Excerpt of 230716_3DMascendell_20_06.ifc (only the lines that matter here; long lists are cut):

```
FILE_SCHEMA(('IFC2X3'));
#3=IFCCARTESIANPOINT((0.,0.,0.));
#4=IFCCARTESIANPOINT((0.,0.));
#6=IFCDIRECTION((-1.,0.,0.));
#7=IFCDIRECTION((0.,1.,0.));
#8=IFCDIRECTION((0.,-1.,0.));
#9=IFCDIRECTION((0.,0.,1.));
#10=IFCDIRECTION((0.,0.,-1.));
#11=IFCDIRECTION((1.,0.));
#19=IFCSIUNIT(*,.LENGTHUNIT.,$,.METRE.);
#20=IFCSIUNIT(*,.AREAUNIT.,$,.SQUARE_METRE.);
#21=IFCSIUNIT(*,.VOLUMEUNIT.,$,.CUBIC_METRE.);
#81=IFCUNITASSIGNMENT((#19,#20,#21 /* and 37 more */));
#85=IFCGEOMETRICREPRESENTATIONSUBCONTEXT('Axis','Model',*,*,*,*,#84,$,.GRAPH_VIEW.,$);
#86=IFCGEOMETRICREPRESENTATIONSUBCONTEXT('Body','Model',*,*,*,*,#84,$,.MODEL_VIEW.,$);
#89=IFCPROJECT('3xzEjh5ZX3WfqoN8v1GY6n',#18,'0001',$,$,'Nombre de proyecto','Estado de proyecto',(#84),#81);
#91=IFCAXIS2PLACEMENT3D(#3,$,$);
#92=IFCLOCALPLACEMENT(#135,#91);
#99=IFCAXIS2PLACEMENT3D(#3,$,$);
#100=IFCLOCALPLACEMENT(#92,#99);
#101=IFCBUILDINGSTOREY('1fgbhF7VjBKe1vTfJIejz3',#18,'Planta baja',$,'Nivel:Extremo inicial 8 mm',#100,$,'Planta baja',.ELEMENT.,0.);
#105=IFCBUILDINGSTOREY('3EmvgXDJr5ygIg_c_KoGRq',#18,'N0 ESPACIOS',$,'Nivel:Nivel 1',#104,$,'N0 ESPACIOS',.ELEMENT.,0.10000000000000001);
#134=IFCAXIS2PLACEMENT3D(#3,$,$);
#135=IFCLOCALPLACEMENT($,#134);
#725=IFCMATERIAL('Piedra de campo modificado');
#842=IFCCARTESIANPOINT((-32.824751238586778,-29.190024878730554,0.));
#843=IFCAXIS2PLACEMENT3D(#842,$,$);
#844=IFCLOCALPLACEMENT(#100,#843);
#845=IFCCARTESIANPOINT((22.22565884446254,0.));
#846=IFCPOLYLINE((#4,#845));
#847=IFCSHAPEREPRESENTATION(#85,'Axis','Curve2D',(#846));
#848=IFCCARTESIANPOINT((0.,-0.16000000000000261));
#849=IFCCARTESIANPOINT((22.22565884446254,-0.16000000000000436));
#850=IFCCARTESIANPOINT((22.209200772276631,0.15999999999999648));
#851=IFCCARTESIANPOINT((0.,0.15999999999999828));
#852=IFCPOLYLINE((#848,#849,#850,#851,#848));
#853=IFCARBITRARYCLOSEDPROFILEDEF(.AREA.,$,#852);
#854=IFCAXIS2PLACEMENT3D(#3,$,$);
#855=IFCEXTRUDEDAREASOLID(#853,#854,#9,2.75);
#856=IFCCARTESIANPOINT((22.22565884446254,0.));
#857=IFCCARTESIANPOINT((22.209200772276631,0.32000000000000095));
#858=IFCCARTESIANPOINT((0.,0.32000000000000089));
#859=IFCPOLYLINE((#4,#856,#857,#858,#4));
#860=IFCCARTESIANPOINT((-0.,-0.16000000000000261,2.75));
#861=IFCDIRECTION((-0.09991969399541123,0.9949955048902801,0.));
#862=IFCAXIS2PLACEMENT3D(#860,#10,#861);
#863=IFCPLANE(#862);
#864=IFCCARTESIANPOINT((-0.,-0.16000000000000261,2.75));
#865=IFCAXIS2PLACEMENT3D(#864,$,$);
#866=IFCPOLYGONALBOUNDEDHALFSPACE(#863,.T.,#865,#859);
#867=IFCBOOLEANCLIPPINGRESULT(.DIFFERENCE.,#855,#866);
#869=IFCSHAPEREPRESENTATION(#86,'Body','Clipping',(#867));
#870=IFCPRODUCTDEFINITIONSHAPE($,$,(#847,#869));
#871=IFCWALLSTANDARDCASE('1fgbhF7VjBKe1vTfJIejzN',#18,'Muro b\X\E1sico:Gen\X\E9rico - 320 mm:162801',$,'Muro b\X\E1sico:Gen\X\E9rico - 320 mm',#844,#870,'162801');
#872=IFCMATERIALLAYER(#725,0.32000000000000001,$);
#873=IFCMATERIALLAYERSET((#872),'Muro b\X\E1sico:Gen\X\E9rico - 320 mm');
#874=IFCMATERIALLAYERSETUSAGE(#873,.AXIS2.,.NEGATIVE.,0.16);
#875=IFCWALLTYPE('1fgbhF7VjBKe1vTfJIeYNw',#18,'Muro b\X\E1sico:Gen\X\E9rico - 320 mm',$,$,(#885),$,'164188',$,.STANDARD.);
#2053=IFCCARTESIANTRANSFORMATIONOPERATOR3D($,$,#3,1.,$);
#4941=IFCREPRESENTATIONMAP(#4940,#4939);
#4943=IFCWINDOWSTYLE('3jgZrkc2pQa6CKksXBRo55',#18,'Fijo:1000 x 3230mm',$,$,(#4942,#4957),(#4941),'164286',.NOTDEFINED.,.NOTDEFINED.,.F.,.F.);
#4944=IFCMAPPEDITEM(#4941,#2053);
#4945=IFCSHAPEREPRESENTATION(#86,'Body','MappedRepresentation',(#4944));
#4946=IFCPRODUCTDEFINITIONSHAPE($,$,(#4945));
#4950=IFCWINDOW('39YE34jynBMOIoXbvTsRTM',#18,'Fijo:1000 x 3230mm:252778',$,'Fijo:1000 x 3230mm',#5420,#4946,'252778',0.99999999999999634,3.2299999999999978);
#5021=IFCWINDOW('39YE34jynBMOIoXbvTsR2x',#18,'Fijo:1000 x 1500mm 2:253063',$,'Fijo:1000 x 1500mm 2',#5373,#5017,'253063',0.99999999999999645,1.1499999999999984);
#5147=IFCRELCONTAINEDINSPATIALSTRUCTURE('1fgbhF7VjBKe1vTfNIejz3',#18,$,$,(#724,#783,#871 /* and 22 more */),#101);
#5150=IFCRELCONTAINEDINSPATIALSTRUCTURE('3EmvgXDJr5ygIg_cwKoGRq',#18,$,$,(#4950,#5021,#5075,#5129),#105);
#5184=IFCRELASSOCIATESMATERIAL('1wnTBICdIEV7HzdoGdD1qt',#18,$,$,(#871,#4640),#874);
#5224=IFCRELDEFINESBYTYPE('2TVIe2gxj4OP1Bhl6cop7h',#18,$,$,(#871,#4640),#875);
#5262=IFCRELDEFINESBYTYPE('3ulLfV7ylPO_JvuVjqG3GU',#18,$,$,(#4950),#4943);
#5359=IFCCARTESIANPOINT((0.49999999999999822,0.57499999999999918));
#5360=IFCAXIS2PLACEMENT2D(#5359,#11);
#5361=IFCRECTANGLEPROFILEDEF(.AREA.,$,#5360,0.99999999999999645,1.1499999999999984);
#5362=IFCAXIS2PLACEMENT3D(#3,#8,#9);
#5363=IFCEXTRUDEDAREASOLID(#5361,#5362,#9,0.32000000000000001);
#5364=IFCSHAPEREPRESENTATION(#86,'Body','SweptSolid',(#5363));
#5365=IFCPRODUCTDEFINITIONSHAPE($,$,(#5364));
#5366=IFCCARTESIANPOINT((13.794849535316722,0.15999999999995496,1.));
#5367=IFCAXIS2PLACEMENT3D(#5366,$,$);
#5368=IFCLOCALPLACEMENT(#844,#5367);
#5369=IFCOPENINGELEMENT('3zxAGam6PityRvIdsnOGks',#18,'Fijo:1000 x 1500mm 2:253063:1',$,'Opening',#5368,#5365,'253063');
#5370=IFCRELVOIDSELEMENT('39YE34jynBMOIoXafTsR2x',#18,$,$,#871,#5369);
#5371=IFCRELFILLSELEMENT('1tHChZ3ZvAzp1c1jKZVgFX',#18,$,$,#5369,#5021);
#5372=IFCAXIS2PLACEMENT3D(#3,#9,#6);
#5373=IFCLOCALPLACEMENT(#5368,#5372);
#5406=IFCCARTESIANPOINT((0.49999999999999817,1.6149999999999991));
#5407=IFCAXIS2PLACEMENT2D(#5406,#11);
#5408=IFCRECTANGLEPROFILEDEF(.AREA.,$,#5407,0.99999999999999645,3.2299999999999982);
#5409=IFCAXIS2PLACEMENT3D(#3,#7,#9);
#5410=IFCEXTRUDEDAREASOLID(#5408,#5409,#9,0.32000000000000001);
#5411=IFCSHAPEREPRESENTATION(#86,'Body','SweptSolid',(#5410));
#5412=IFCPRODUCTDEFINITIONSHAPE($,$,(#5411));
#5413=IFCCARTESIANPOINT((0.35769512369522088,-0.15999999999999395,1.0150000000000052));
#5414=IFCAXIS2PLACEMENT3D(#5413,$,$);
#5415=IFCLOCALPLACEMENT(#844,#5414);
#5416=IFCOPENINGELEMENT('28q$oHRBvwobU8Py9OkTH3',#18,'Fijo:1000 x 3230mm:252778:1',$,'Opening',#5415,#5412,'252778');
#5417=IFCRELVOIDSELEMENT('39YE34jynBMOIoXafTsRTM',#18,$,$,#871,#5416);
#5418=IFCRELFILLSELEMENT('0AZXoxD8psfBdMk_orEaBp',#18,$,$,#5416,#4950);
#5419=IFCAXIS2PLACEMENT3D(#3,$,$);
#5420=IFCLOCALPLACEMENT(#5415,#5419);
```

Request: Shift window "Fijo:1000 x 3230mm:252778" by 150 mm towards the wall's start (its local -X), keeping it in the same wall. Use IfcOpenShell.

```python
import ifcopenshell
import ifcopenshell.api.geometry
import ifcopenshell.util.placement
import ifcopenshell.util.unit

model = ifcopenshell.open("230716_3DMascendell_20_06.ifc")
unit_scale = ifcopenshell.util.unit.calculate_unit_scale(model)

window = model.by_guid("39YE34jynBMOIoXbvTsRTM")
opening = window.FillsVoids[0].RelatingOpeningElement
wall = opening.VoidsElements[0].RelatingBuildingElement

wall_matrix = ifcopenshell.util.placement.get_local_placement(wall.ObjectPlacement)
shift = wall_matrix[:3, 0] * -0.15 / unit_scale
before = ifcopenshell.util.placement.get_local_placement(window.ObjectPlacement)[:3, 3].copy()

# The window is placed relative to its opening, so it follows when the opening moves.
matrix = ifcopenshell.util.placement.get_local_placement(opening.ObjectPlacement)
matrix[:3, 3] += shift
ifcopenshell.api.geometry.edit_object_placement(
    model, product=opening, matrix=matrix, is_si=False, should_transform_children=True
)

after = ifcopenshell.util.placement.get_local_placement(window.ObjectPlacement)[:3, 3]
print("window moved by", (after - before).round(3) + 0.0)

model.write("230716_3DMascendell_20_06_updated.ifc")
```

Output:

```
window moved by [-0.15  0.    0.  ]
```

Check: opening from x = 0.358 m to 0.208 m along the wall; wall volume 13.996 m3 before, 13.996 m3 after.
